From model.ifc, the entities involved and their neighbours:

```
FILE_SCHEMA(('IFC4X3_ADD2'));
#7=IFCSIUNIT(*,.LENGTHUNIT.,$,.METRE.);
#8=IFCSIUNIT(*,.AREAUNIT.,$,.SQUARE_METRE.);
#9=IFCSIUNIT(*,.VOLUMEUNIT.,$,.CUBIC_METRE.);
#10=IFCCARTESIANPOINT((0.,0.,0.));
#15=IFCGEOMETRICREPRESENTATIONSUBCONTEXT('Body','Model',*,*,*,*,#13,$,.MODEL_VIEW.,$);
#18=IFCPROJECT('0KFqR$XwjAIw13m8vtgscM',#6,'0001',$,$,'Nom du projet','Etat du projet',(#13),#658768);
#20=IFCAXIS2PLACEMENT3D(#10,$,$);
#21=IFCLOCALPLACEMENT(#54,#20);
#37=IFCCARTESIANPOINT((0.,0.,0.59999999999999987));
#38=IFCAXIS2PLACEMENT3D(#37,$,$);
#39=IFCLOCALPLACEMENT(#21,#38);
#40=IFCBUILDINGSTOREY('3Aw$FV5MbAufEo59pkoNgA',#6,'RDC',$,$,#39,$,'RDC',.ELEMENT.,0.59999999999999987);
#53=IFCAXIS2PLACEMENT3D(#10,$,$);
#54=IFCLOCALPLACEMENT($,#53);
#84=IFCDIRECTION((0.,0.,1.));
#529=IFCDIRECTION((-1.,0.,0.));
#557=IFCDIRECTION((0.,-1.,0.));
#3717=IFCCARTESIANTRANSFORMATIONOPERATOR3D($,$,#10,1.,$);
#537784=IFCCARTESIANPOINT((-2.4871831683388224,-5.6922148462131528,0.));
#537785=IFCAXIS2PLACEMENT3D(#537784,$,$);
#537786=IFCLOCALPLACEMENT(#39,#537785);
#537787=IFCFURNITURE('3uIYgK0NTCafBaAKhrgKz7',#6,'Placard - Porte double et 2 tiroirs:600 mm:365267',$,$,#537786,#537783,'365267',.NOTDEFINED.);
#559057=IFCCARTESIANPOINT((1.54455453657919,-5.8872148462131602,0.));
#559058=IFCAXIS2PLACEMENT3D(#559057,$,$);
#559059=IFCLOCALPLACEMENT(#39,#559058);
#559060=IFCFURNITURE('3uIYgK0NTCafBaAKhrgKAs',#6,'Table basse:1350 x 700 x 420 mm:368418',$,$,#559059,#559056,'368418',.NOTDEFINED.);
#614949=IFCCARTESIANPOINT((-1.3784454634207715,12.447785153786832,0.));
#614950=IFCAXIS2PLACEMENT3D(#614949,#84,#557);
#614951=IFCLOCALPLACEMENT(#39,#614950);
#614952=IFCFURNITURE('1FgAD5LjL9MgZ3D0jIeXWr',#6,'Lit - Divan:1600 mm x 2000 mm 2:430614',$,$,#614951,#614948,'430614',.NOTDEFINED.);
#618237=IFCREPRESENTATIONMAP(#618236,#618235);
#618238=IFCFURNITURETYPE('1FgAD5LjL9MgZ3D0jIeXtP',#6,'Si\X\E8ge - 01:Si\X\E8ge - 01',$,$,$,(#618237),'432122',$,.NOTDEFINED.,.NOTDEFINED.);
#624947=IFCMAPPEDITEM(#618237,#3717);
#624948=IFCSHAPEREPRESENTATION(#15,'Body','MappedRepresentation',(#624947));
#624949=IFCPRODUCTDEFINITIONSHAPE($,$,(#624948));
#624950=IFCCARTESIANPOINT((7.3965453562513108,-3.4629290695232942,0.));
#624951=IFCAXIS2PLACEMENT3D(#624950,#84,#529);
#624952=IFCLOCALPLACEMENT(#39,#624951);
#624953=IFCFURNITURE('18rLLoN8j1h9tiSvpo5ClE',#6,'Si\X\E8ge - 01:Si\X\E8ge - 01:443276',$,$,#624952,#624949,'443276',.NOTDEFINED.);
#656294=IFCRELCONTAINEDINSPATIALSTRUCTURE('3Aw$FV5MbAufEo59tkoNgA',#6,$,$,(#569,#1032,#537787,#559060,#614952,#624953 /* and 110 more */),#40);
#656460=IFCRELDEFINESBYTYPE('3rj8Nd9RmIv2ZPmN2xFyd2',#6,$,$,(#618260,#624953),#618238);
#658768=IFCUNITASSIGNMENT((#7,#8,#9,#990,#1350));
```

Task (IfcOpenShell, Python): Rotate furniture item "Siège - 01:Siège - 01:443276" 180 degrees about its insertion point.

```python
import ifcopenshell
import ifcopenshell.api.geometry
import ifcopenshell.util.placement

model = ifcopenshell.open("model.ifc")

item = model.by_guid("18rLLoN8j1h9tiSvpo5ClE")
matrix = ifcopenshell.util.placement.get_local_placement(item.ObjectPlacement)
matrix = matrix @ ifcopenshell.util.placement.rotation(180, "Z")
ifcopenshell.api.geometry.edit_object_placement(model, product=item, matrix=matrix, is_si=False)

print(ifcopenshell.util.placement.get_local_placement(item.ObjectPlacement).round(3) + 0.0)

model.write("model_v2.ifc")
```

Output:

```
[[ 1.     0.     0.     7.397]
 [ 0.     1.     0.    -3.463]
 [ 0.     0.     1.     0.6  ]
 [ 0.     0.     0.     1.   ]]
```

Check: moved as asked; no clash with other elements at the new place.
